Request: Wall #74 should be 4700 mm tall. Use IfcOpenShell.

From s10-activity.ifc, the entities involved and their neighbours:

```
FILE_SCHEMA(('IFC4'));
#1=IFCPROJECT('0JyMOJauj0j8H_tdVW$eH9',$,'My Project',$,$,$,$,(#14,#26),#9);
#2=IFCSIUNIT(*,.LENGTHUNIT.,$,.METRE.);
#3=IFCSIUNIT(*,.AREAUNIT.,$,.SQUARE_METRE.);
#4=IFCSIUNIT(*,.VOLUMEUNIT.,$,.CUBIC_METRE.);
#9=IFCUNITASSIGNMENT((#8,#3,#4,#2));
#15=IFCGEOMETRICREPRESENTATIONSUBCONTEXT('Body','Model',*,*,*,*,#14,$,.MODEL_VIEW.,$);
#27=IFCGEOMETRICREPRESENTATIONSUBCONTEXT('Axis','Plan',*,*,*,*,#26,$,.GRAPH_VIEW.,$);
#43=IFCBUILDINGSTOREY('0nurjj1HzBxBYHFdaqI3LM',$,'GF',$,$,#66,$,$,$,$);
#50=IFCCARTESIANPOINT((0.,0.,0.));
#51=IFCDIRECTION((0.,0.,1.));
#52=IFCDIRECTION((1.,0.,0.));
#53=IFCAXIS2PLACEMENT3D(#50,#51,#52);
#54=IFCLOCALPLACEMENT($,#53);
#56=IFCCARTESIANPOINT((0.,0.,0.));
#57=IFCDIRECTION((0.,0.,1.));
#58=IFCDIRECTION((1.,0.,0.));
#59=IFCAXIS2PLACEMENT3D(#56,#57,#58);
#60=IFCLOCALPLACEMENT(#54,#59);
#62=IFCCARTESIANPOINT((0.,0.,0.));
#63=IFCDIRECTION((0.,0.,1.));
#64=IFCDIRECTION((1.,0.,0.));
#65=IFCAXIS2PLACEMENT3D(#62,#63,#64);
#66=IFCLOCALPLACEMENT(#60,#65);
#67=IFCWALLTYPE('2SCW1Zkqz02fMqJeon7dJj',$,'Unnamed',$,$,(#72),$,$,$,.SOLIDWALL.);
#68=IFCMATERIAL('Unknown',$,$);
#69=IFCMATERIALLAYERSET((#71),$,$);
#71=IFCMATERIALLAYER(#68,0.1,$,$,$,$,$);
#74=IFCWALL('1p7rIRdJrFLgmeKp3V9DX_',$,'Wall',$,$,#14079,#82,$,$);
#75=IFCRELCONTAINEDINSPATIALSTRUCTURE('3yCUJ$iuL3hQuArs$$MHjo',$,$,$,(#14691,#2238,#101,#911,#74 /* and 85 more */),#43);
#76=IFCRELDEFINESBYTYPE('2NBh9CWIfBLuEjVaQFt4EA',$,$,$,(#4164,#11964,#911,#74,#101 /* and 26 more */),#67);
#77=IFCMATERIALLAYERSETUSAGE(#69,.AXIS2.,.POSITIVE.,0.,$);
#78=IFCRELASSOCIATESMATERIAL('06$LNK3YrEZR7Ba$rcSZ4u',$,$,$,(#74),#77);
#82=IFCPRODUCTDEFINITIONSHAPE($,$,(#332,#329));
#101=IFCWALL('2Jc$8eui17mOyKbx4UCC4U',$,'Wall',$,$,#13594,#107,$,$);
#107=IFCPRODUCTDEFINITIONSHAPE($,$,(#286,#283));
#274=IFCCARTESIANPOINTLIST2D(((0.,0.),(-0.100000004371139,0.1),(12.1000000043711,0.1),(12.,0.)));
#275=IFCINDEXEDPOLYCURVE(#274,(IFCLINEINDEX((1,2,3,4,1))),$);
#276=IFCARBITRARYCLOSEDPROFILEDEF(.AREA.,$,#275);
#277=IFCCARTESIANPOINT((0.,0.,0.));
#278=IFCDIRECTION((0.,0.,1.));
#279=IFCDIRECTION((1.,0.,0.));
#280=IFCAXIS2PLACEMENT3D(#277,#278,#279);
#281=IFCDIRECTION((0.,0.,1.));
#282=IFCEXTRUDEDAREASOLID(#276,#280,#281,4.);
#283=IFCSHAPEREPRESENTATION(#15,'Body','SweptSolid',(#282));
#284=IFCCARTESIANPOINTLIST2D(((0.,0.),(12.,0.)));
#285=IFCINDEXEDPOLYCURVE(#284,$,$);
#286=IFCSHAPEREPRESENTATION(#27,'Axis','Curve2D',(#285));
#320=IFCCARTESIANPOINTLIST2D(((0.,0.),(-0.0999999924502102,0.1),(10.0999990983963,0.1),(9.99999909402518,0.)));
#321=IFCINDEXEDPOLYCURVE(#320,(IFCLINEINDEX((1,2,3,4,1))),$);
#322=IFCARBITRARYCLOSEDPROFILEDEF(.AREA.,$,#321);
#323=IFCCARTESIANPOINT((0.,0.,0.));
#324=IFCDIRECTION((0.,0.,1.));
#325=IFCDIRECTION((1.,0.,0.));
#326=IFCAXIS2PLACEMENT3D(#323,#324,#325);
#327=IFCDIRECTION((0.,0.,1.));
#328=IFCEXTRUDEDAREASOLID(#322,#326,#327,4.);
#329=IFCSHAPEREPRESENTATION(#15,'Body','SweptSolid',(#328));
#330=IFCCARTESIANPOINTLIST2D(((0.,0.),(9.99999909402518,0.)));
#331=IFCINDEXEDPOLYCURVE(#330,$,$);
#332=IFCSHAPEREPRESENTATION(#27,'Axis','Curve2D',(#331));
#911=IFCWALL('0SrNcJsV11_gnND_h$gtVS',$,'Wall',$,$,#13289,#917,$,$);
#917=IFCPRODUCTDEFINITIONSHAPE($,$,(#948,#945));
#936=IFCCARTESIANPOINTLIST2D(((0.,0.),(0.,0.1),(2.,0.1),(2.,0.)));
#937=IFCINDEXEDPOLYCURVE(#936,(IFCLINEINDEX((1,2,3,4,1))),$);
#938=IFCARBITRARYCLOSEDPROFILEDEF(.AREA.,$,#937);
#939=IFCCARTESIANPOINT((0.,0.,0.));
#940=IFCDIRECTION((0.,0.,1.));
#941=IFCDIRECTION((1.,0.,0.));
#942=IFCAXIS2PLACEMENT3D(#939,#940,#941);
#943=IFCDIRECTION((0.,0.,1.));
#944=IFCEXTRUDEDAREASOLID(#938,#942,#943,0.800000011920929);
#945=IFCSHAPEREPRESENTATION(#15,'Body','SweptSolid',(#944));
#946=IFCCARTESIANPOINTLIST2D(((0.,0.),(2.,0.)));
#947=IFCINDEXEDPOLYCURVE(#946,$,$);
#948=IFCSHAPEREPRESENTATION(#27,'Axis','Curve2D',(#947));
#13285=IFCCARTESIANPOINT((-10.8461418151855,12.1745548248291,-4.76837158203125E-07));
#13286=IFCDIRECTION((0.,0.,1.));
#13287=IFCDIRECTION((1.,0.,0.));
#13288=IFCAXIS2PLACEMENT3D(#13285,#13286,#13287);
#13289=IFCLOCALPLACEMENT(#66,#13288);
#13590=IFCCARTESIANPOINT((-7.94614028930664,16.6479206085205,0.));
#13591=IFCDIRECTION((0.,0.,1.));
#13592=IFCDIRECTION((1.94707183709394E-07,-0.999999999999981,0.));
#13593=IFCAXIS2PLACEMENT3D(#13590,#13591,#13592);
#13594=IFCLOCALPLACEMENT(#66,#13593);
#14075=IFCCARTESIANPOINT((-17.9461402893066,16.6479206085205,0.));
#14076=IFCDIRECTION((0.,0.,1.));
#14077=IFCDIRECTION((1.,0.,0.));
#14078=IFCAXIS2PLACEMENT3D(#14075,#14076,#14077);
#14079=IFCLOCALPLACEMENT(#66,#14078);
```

```python
import ifcopenshell
import ifcopenshell.geom
import ifcopenshell.util.representation
import ifcopenshell.util.shape
import ifcopenshell.util.unit

model = ifcopenshell.open("s10-activity.ifc")
unit_scale = ifcopenshell.util.unit.calculate_unit_scale(model)
settings = ifcopenshell.geom.settings()


def volume(element):
    """Net volume in cubic metres, openings subtracted."""
    shape = ifcopenshell.geom.create_shape(settings, element)
    return ifcopenshell.util.shape.get_volume(shape.geometry)


wall = model.by_guid("1p7rIRdJrFLgmeKp3V9DX_")
before = volume(wall)

body = ifcopenshell.util.representation.get_representation(wall, "Model", "Body")
solid = body.Items[0]
old_height = solid.Depth
solid.Depth = 4.7 / unit_scale
after = volume(wall)

print(f"height {old_height:g} -> {solid.Depth:g}, volume {before:.3f} -> {after:.3f} m3")

model.write("s10-activity-out.ifc")
```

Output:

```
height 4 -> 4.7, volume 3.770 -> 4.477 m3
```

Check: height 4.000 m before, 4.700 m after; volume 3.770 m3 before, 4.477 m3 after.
